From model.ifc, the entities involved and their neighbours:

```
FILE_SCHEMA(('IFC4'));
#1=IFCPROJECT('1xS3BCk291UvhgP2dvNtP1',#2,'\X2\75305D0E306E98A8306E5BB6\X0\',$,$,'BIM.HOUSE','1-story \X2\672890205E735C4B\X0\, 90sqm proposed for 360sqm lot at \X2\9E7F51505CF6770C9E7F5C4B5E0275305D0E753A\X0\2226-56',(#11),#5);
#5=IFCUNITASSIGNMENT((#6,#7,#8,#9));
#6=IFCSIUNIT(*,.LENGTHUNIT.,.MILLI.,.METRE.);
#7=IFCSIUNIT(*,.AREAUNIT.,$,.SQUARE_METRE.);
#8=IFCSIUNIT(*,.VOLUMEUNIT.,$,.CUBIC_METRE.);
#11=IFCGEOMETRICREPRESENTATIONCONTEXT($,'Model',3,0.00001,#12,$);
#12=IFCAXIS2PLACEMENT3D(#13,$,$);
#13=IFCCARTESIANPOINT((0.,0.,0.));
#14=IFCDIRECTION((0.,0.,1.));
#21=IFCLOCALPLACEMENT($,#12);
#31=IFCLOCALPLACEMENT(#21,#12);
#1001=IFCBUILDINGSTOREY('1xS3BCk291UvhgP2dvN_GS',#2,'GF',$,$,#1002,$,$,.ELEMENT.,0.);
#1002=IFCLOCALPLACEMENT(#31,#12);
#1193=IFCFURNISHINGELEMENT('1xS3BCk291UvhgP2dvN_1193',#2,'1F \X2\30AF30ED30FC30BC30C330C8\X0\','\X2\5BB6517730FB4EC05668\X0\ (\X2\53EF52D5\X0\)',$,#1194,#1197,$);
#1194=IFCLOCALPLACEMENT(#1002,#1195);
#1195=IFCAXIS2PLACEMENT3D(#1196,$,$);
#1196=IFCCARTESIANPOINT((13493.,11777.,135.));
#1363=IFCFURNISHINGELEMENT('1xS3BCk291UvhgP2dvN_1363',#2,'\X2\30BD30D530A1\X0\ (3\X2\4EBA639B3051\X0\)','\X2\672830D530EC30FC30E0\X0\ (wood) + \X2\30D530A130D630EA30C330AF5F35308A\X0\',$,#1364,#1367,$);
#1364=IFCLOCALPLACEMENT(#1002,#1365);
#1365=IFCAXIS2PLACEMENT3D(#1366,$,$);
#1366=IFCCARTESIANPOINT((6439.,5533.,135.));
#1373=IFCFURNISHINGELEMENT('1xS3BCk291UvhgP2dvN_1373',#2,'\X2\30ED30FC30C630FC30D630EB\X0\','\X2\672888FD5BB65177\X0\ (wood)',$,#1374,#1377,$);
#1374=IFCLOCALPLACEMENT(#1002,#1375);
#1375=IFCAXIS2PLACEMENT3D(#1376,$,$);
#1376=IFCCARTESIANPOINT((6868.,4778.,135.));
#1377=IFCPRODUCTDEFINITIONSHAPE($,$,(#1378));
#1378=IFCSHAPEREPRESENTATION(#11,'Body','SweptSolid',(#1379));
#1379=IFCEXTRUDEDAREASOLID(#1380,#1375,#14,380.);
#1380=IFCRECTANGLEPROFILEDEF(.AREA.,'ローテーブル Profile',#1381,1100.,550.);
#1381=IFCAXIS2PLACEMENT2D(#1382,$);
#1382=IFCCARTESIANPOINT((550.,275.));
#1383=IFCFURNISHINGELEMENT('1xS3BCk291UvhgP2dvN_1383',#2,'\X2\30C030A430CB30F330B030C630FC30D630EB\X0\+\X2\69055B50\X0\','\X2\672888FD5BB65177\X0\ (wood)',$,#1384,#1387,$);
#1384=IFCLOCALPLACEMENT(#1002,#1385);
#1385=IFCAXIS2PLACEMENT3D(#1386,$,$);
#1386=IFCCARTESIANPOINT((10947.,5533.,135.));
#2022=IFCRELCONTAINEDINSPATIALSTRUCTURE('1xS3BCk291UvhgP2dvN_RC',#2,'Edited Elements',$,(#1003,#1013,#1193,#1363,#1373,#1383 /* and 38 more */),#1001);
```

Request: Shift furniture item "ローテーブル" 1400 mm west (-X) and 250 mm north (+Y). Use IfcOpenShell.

```python
import ifcopenshell
import ifcopenshell.api.geometry
import ifcopenshell.util.placement
import ifcopenshell.util.unit

model = ifcopenshell.open("model.ifc")
unit_scale = ifcopenshell.util.unit.calculate_unit_scale(model)

item = model.by_id(1373)
matrix = ifcopenshell.util.placement.get_local_placement(item.ObjectPlacement)
matrix[0, 3] -= 1.4 / unit_scale
matrix[1, 3] += 0.25 / unit_scale
ifcopenshell.api.geometry.edit_object_placement(model, product=item, matrix=matrix, is_si=False)

print(ifcopenshell.util.placement.get_local_placement(item.ObjectPlacement).round(3) + 0.0)

model.write("model_updated.ifc")
```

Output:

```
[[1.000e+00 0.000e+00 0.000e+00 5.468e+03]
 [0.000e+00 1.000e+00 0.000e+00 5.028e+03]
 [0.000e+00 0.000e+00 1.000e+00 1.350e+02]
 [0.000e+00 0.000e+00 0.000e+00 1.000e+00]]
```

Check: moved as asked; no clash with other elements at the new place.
